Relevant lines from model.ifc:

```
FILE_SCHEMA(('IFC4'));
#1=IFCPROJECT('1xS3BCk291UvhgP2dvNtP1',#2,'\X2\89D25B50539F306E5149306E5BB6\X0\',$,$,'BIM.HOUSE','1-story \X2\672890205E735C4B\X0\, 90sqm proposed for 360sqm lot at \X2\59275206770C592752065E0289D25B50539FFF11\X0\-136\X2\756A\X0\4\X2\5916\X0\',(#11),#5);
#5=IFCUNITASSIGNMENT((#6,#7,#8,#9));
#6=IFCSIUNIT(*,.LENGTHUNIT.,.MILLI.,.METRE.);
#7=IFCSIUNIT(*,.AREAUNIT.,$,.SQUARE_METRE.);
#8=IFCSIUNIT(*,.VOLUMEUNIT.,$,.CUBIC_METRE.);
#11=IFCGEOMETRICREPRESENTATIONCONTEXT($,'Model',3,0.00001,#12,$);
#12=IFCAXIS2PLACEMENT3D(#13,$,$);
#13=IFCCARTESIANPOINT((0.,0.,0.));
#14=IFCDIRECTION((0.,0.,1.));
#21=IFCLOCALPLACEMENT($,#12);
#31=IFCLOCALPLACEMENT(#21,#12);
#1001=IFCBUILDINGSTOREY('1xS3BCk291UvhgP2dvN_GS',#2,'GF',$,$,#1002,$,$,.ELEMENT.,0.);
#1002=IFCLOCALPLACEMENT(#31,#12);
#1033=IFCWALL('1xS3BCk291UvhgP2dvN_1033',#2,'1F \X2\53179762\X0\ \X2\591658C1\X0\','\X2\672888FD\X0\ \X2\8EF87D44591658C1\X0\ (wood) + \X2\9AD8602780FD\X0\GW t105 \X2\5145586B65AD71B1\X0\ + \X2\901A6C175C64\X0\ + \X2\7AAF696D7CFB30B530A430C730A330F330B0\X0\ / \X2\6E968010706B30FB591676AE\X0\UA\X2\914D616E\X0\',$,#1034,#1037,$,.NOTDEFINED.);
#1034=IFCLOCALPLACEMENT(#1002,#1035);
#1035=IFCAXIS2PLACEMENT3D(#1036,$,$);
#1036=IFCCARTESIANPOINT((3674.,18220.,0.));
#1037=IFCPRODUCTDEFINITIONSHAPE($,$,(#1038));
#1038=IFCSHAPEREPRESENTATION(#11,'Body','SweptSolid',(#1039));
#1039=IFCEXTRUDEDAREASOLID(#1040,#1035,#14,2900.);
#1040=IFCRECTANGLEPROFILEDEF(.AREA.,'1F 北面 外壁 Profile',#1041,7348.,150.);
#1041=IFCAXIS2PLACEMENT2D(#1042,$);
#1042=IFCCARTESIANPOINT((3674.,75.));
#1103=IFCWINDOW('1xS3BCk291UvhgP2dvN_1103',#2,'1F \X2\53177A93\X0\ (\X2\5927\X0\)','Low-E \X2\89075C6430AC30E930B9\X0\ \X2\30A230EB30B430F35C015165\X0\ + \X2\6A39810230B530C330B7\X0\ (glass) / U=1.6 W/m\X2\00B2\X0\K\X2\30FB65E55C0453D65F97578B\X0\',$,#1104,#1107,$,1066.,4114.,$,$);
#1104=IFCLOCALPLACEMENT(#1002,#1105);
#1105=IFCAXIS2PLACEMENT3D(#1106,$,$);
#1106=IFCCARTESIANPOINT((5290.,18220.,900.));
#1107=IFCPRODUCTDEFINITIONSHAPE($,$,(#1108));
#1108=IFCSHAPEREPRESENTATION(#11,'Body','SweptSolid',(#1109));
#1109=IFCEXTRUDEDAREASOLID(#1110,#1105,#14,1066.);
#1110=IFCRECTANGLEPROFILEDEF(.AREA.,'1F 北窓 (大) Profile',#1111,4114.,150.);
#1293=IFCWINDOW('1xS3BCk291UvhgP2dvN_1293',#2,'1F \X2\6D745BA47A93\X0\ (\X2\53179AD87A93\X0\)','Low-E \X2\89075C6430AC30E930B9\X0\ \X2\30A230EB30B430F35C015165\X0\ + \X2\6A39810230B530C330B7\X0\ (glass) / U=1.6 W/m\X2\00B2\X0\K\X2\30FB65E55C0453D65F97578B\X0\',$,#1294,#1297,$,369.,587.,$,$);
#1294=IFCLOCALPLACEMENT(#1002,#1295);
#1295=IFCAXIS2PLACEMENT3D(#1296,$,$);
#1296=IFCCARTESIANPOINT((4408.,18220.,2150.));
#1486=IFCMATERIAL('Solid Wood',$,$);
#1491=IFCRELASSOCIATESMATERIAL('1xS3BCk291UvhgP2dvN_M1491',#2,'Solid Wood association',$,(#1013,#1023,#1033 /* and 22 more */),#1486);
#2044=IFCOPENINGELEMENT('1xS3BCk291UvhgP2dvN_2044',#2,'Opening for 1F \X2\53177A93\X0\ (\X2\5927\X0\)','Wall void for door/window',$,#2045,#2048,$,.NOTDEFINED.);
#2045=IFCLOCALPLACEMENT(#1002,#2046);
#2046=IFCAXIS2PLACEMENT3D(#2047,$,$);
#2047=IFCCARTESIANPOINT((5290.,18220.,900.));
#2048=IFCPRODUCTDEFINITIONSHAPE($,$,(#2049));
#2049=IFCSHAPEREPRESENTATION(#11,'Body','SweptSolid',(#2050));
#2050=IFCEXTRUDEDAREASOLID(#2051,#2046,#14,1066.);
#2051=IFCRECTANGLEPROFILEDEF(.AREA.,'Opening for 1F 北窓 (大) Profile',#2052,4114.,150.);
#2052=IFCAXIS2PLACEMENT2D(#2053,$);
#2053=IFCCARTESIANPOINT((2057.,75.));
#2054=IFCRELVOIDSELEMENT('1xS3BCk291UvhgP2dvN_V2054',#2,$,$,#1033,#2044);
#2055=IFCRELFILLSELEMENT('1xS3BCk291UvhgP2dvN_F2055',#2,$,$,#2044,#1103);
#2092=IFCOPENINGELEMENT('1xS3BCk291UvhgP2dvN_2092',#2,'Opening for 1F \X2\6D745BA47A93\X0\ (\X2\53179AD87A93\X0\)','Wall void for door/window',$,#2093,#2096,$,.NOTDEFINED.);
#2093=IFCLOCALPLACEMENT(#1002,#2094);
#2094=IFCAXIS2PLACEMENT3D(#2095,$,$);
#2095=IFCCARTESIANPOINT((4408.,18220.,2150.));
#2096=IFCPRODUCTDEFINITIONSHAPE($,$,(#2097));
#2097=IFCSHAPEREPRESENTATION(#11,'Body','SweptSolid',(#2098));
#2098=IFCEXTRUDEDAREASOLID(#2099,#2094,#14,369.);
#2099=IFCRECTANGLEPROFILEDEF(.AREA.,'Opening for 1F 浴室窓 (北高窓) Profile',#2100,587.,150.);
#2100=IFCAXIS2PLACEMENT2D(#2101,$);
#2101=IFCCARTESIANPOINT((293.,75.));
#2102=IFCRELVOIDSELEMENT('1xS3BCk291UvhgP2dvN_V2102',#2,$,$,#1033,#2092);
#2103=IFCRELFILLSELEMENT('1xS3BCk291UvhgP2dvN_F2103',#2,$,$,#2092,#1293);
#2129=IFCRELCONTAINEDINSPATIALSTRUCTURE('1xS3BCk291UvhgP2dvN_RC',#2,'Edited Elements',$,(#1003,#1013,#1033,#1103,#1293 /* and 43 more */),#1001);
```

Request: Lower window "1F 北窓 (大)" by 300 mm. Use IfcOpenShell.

```python
import numpy as np
import ifcopenshell
import ifcopenshell.api.geometry
import ifcopenshell.util.placement
import ifcopenshell.util.unit

model = ifcopenshell.open("model.ifc")
unit_scale = ifcopenshell.util.unit.calculate_unit_scale(model)

window = model.by_id(1103)
opening = window.FillsVoids[0].RelatingOpeningElement
dz = -0.3 / unit_scale

shift = np.array([0.0, 0.0, dz])
# The window is not placed relative to its opening, so move both.
for product in (opening, window):
    matrix = ifcopenshell.util.placement.get_local_placement(product.ObjectPlacement)
    matrix[:3, 3] += shift
    ifcopenshell.api.geometry.edit_object_placement(model, product=product, matrix=matrix, is_si=False)

print(f"moved by {dz * unit_scale:+.3f} m")

model.write("model_v2.ifc")
```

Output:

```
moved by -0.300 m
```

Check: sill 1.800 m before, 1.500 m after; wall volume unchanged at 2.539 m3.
